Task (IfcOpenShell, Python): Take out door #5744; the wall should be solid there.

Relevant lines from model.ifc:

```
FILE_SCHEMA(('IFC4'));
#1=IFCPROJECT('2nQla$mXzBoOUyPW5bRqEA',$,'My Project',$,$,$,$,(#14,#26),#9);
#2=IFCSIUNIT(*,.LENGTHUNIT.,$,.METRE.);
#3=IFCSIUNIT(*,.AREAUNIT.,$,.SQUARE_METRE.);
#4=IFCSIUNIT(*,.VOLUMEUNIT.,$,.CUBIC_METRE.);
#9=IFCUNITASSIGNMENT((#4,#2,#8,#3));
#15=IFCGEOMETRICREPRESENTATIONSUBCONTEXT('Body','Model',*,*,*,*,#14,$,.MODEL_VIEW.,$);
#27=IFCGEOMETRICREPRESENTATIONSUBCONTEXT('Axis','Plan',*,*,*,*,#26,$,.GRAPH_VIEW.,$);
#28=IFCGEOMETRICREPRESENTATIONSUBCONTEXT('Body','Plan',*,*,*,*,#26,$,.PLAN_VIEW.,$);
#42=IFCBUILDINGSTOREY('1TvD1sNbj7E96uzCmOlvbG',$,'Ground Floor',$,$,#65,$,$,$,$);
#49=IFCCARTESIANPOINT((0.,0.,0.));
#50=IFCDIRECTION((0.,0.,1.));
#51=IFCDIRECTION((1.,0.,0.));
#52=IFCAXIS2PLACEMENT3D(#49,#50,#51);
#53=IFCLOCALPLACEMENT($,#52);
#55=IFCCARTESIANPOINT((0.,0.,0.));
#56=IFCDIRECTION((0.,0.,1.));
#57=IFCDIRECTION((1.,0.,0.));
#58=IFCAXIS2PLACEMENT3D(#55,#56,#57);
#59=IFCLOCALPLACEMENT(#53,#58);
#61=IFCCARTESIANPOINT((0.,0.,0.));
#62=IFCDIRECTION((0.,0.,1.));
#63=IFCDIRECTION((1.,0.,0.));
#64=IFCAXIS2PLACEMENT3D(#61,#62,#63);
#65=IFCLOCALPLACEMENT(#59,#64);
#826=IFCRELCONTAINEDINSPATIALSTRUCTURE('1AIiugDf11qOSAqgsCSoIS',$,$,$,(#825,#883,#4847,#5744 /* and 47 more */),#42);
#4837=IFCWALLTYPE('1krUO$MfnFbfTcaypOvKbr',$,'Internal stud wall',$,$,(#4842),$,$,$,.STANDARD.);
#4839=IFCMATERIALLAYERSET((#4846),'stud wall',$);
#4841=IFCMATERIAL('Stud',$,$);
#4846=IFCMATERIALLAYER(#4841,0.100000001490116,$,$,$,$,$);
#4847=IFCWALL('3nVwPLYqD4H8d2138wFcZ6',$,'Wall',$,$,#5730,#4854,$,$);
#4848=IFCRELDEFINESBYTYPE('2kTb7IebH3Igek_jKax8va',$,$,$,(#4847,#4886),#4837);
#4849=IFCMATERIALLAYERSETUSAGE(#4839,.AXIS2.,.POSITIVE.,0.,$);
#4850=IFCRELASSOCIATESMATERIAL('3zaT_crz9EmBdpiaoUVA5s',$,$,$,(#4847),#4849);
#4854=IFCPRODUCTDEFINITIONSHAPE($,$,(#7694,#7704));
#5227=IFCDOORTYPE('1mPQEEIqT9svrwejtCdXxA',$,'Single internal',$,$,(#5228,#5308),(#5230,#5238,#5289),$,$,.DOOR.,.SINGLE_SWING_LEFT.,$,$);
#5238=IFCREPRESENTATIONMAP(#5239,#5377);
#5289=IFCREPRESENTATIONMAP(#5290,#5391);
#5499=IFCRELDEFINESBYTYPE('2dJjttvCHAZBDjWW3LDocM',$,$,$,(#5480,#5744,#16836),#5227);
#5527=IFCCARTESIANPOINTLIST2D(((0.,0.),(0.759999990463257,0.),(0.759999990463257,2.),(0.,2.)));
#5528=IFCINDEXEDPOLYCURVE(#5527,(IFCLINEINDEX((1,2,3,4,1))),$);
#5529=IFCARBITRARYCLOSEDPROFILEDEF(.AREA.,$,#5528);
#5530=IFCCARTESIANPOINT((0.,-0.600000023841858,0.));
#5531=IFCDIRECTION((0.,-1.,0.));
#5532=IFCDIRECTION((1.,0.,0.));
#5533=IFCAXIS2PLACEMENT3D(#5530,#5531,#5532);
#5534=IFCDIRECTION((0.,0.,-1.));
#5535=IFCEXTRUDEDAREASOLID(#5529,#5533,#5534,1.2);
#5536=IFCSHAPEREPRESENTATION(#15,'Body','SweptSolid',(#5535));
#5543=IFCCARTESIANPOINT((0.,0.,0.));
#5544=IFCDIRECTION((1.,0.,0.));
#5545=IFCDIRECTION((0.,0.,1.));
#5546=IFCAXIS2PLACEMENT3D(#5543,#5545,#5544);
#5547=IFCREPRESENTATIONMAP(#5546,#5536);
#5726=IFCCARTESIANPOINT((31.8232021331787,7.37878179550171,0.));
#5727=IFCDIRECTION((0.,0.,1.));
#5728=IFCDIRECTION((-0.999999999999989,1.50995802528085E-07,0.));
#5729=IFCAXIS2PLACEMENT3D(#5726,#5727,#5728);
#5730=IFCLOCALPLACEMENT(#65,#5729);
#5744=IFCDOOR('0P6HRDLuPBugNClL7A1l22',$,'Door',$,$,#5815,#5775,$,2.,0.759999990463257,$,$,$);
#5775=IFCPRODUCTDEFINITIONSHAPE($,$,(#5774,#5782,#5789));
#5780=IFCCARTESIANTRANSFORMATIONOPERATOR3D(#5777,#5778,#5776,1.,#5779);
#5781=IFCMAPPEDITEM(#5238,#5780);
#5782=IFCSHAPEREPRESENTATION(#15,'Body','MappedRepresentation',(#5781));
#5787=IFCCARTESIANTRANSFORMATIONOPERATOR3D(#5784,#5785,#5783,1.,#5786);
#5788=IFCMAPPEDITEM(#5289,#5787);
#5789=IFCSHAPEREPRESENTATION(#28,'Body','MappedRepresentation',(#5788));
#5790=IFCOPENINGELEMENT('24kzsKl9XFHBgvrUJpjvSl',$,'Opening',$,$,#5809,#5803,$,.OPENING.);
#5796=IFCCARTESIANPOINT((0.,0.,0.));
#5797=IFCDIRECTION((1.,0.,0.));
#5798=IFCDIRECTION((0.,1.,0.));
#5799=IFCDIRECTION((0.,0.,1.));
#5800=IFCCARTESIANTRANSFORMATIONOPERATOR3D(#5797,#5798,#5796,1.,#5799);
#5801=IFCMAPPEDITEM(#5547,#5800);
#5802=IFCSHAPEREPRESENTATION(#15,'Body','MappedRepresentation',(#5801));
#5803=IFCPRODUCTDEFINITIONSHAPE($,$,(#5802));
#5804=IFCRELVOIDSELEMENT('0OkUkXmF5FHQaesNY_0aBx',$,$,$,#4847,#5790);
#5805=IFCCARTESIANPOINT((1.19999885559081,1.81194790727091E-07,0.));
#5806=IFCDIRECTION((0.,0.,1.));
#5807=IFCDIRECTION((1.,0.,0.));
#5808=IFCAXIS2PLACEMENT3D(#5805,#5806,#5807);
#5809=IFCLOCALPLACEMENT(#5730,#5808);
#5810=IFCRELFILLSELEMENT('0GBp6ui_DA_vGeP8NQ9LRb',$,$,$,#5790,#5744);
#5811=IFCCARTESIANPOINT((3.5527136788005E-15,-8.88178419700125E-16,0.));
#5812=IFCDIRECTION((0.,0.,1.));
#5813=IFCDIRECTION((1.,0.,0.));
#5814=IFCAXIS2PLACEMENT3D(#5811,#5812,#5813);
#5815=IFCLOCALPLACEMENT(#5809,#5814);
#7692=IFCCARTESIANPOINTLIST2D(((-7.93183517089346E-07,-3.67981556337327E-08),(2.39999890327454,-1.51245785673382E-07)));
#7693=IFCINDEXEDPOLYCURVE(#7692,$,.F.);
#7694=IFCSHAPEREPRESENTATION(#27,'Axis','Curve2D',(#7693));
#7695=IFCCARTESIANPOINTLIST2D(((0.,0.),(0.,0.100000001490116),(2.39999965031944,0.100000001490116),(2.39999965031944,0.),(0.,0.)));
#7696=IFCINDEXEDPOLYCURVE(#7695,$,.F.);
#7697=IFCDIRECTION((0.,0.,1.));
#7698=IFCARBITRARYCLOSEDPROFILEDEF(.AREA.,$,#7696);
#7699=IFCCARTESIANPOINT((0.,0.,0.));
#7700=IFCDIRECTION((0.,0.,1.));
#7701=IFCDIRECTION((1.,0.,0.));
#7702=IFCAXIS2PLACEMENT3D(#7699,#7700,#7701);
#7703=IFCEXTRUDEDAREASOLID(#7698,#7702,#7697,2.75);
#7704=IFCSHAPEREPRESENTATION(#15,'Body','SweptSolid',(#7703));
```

```python
import ifcopenshell
import ifcopenshell.api.feature
import ifcopenshell.api.root
import ifcopenshell.geom
import ifcopenshell.util.shape

model = ifcopenshell.open("model.ifc")
settings = ifcopenshell.geom.settings()


def volume(element):
    """Net volume in cubic metres, openings subtracted."""
    shape = ifcopenshell.geom.create_shape(settings, element)
    return ifcopenshell.util.shape.get_volume(shape.geometry)


door = model.by_guid("0P6HRDLuPBugNClL7A1l22")
opening = door.FillsVoids[0].RelatingOpeningElement
wall = opening.VoidsElements[0].RelatingBuildingElement
before = volume(wall)

ifcopenshell.api.root.remove_product(model, product=door)
ifcopenshell.api.feature.remove_feature(model, feature=opening)

after = volume(wall)

print(f"wall volume {before:.3f} -> {after:.3f} m3")

model.write("model_edited.ifc")
```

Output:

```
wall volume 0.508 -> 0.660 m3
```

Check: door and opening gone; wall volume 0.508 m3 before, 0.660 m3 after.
